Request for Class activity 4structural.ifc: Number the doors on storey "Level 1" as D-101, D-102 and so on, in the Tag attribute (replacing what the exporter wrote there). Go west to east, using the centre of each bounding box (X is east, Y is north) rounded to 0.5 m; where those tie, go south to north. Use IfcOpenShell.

First a look at what the model holds.

```python
import ifcopenshell
import ifcopenshell.util.element
import ifcopenshell.util.placement

model = ifcopenshell.open("Class activity 4structural.ifc")
print(model.schema)
storey = next(s for s in model.by_type("IfcBuildingStorey") if s.Name == "Level 1")
doors = [e for e in ifcopenshell.util.element.get_decomposition(storey) if e.is_a("IfcDoor")]
for e in sorted(doors, key=lambda e: e.id()):
    origin = ifcopenshell.util.placement.get_local_placement(e.ObjectPlacement)[:3, 3]
    print(e.id(), e.Tag, e.Name, origin.round(2) + 0.0, sep=" | ")
```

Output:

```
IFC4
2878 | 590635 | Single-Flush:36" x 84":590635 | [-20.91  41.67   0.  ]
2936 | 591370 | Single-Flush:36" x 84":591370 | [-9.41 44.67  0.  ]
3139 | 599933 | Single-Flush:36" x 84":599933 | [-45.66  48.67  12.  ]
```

```python
import ifcopenshell
import ifcopenshell.geom
import ifcopenshell.util.element
import ifcopenshell.util.shape

model = ifcopenshell.open("Class activity 4structural.ifc")
settings = ifcopenshell.geom.settings()
settings.set("use-world-coords", True)


def centre(element):
    shape = ifcopenshell.geom.create_shape(settings, element)
    return ifcopenshell.util.shape.get_bbox_centroid(shape.geometry)


storey = next(s for s in model.by_type("IfcBuildingStorey") if s.Name == "Level 1")
doors = [e for e in ifcopenshell.util.element.get_decomposition(storey) if e.is_a("IfcDoor")]

# Insertion points can sit at a corner or the storey origin, so sort by the geometry (in metres).
centres = {e: centre(e) for e in doors}
doors.sort(key=lambda e: (round(centres[e][0] / 0.5), centres[e][1]))

for i, e in enumerate(doors, start=1):
    number = f"D-1{i:02d}"
    e.Tag = number
    print(e.id(), number)

model.write("Class activity 4structural_updated.ifc")
```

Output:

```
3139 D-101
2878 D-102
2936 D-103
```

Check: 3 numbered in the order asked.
